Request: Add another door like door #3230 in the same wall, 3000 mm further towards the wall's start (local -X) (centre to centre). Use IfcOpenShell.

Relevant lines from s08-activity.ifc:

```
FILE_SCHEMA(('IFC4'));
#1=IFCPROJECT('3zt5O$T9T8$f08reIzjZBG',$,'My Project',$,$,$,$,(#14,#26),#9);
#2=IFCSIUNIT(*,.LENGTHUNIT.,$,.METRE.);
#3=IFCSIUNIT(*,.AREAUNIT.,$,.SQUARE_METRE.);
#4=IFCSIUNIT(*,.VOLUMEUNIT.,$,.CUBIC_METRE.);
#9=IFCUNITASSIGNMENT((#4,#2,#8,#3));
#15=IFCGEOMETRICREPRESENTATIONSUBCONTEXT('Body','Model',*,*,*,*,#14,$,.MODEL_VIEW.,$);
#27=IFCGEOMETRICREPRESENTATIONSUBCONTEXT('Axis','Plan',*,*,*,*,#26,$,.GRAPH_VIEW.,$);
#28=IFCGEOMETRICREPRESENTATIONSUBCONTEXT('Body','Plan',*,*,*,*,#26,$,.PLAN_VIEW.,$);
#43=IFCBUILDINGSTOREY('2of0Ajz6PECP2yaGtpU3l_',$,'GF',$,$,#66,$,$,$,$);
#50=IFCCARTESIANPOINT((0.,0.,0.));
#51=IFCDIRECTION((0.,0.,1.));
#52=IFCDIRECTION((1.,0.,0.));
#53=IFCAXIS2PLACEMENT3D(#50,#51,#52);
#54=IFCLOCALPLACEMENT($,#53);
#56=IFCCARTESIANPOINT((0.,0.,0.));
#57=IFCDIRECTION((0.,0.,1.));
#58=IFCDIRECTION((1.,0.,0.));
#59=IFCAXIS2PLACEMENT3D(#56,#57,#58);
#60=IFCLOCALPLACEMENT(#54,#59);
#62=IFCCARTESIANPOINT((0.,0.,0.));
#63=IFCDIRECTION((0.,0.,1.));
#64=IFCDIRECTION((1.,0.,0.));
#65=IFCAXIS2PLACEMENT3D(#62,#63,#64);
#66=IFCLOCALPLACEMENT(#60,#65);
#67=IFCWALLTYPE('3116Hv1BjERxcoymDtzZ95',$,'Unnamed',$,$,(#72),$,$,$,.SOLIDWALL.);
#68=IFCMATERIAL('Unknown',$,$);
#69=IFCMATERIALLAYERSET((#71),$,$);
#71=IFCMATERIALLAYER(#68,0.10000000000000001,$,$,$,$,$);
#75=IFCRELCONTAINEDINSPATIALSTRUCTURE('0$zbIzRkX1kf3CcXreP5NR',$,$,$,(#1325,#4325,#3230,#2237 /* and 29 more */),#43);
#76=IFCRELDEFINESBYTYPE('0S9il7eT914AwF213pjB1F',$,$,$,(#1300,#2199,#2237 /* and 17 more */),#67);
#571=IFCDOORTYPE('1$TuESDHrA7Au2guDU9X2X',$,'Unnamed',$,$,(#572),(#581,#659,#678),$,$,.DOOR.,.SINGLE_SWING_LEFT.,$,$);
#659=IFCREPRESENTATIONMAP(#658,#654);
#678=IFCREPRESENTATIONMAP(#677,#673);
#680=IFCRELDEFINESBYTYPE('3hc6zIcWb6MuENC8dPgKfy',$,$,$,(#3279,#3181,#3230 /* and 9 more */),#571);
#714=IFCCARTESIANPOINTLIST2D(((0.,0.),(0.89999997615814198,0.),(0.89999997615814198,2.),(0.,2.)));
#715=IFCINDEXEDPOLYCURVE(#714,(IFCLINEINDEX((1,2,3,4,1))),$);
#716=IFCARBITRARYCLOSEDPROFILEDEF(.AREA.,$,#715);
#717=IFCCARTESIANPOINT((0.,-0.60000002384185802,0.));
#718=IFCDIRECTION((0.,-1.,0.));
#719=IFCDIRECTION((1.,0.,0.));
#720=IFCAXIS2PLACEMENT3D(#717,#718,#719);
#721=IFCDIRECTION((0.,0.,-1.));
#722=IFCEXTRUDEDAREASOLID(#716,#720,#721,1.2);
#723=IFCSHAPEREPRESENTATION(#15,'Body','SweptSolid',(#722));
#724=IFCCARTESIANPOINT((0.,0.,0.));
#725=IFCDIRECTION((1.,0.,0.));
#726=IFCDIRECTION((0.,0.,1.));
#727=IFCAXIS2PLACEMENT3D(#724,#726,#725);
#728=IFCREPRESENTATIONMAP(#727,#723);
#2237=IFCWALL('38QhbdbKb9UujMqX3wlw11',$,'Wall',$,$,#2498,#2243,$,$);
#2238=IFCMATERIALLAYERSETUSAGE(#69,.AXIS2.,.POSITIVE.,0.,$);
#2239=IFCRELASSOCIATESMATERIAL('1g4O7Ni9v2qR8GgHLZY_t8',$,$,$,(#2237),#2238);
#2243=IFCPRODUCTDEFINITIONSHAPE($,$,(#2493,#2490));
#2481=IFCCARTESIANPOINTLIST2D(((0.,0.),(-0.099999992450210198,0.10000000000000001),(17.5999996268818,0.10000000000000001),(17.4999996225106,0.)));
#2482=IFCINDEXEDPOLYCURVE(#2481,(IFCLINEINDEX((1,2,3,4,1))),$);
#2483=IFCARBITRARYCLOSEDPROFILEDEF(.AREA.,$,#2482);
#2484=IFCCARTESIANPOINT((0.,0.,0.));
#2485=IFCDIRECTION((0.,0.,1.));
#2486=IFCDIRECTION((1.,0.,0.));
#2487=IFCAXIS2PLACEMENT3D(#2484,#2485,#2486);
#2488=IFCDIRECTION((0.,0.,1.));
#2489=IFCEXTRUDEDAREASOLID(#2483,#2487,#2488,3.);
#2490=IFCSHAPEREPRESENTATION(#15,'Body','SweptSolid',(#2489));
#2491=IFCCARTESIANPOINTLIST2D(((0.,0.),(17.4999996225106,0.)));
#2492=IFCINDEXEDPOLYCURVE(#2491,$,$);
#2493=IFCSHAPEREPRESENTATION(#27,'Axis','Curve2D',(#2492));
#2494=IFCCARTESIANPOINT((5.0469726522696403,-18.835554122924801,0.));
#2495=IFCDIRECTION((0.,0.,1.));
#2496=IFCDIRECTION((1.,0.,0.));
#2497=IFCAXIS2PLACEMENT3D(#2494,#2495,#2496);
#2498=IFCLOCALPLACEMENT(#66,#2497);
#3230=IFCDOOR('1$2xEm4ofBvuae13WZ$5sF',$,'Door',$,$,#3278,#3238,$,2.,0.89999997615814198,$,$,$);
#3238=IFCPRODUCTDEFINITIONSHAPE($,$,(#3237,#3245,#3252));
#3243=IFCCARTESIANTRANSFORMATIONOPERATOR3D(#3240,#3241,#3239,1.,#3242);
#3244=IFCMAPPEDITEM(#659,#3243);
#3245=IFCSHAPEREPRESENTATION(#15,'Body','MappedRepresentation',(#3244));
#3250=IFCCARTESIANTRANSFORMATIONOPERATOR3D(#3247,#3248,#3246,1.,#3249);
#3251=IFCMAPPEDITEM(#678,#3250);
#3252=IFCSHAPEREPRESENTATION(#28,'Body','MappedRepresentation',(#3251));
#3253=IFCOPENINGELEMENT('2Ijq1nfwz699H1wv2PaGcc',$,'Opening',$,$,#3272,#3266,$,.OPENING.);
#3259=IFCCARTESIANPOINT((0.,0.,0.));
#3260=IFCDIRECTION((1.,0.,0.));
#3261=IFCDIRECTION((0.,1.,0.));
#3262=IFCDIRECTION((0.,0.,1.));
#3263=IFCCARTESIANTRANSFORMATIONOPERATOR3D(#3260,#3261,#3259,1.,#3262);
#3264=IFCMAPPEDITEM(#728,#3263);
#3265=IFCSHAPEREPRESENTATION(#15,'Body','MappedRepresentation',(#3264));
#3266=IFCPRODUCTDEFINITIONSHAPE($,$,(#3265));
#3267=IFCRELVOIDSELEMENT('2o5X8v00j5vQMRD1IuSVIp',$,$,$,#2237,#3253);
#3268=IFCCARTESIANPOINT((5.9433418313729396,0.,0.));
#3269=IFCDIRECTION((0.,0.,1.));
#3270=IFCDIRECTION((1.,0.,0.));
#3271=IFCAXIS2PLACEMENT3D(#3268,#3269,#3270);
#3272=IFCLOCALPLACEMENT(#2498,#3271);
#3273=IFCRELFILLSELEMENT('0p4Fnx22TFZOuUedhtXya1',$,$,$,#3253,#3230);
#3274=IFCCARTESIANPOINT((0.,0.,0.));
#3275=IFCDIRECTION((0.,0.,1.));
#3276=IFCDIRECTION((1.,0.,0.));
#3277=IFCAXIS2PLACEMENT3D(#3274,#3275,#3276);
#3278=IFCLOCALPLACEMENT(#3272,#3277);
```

```python
import ifcopenshell
import ifcopenshell.api.feature
import ifcopenshell.api.geometry
import ifcopenshell.api.root
import ifcopenshell.geom
import ifcopenshell.util.element
import ifcopenshell.util.placement
import ifcopenshell.util.shape

model = ifcopenshell.open("s08-activity.ifc")
settings = ifcopenshell.geom.settings()


def volume(element):
    """Net volume in cubic metres, openings subtracted."""
    shape = ifcopenshell.geom.create_shape(settings, element)
    return ifcopenshell.util.shape.get_volume(shape.geometry)


door = model.by_id(3230)
opening = door.FillsVoids[0].RelatingOpeningElement
wall = opening.VoidsElements[0].RelatingBuildingElement
before = volume(wall)
shift = ifcopenshell.util.placement.get_local_placement(wall.ObjectPlacement)[:3, 0] * -3.0

# copy_class copies the void relationship, type, container and properties, but no geometry.
new_opening = ifcopenshell.api.root.copy_class(model, product=opening)
new_opening.Representation = ifcopenshell.util.element.copy_deep(
    model, opening.Representation, exclude=["IfcGeometricRepresentationContext", "IfcRepresentationMap"]
)
new_door = ifcopenshell.api.root.copy_class(model, product=door)
new_door.Representation = ifcopenshell.util.element.copy_deep(
    model, door.Representation, exclude=["IfcGeometricRepresentationContext", "IfcRepresentationMap"]
)
ifcopenshell.api.feature.add_filling(model, opening=new_opening, element=new_door)

for old, new in ((opening, new_opening), (door, new_door)):
    matrix = ifcopenshell.util.placement.get_local_placement(old.ObjectPlacement)
    matrix[:3, 3] += shift
    ifcopenshell.api.geometry.edit_object_placement(model, product=new, matrix=matrix, is_si=False)

after = volume(wall)

print(f"wall volume {before:.3f} -> {after:.3f} m3")

model.write("s08-activity-out.ifc")
```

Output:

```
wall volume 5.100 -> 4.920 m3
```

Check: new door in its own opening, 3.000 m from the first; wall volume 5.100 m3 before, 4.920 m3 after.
